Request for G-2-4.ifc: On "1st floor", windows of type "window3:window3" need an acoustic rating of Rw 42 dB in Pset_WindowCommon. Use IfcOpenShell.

First a look at what the model holds.

```python
import ifcopenshell
import ifcopenshell.util.element

model = ifcopenshell.open("G-2-4.ifc")
print(model.schema)
storey = next(s for s in model.by_type("IfcBuildingStorey") if s.Name == "1st floor")
windows = [e for e in ifcopenshell.util.element.get_decomposition(storey) if e.is_a("IfcWindow")]
seen = {}
for e in windows:
    element_type = ifcopenshell.util.element.get_type(e)
    key = (element_type.Name if element_type != e and element_type else None, ifcopenshell.util.element.get_pset(e, "Pset_WindowCommon", "AcousticRating"))
    seen[key] = seen.get(key, 0) + 1
for (name, value), count in sorted(seen.items(), key=str):
    print(count, "x", name, "|", value)
```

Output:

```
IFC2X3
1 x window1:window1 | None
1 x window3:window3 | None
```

```python
import ifcopenshell
import ifcopenshell.api.pset
import ifcopenshell.util.element

model = ifcopenshell.open("G-2-4.ifc")

storey = next(s for s in model.by_type("IfcBuildingStorey") if s.Name == "1st floor")
windows = [e for e in ifcopenshell.util.element.get_decomposition(storey) if e.is_a("IfcWindow")]

count = 0
for e in windows:
    element_type = ifcopenshell.util.element.get_type(e)
    if element_type in (None, e) or element_type.Name != "window3:window3":
        continue
    # add_pset returns the element's existing set when there is one.
    pset = ifcopenshell.api.pset.add_pset(model, product=e, name="Pset_WindowCommon")
    ifcopenshell.api.pset.edit_pset(model, pset=pset, properties={"AcousticRating": "Rw 42 dB"})
    count += 1

print(count, "windows updated")

model.write("G-2-4_edited.ifc")
```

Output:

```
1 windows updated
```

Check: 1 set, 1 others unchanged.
